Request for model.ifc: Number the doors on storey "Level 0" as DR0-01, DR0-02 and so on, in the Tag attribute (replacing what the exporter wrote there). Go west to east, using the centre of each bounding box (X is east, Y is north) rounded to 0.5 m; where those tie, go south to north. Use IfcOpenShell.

First a look at what the model holds.

```python
import ifcopenshell
import ifcopenshell.util.element
import ifcopenshell.util.placement

model = ifcopenshell.open("model.ifc")
print(model.schema)
storey = next(s for s in model.by_type("IfcBuildingStorey") if s.Name == "Level 0")
doors = [e for e in ifcopenshell.util.element.get_decomposition(storey) if e.is_a("IfcDoor")]
for e in sorted(doors, key=lambda e: e.id()):
    origin = ifcopenshell.util.placement.get_local_placement(e.ObjectPlacement)[:3, 3]
    print(e.id(), e.Tag, e.Name, origin.round(2) + 0.0, sep=" | ")
```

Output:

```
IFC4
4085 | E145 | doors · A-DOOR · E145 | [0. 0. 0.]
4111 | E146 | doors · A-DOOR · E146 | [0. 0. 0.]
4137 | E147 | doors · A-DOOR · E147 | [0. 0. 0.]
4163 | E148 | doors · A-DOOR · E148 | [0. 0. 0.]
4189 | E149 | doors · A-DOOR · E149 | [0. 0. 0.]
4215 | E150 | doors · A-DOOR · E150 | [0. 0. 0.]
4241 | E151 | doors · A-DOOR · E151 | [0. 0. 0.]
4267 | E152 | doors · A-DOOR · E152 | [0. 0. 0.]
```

```python
import ifcopenshell
import ifcopenshell.geom
import ifcopenshell.util.element
import ifcopenshell.util.shape

model = ifcopenshell.open("model.ifc")
settings = ifcopenshell.geom.settings()
settings.set("use-world-coords", True)


def centre(element):
    shape = ifcopenshell.geom.create_shape(settings, element)
    return ifcopenshell.util.shape.get_bbox_centroid(shape.geometry)


storey = next(s for s in model.by_type("IfcBuildingStorey") if s.Name == "Level 0")
doors = [e for e in ifcopenshell.util.element.get_decomposition(storey) if e.is_a("IfcDoor")]

# Insertion points can sit at a corner or the storey origin, so sort by the geometry (in metres).
centres = {e: centre(e) for e in doors}
doors.sort(key=lambda e: (round(centres[e][0] / 0.5), centres[e][1]))

for i, e in enumerate(doors, start=1):
    number = f"DR0-{i:02d}"
    e.Tag = number
    print(e.id(), number)

model.write("model_v2.ifc")
```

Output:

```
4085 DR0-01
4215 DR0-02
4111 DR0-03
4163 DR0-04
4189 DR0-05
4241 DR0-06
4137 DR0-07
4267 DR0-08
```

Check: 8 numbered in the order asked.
